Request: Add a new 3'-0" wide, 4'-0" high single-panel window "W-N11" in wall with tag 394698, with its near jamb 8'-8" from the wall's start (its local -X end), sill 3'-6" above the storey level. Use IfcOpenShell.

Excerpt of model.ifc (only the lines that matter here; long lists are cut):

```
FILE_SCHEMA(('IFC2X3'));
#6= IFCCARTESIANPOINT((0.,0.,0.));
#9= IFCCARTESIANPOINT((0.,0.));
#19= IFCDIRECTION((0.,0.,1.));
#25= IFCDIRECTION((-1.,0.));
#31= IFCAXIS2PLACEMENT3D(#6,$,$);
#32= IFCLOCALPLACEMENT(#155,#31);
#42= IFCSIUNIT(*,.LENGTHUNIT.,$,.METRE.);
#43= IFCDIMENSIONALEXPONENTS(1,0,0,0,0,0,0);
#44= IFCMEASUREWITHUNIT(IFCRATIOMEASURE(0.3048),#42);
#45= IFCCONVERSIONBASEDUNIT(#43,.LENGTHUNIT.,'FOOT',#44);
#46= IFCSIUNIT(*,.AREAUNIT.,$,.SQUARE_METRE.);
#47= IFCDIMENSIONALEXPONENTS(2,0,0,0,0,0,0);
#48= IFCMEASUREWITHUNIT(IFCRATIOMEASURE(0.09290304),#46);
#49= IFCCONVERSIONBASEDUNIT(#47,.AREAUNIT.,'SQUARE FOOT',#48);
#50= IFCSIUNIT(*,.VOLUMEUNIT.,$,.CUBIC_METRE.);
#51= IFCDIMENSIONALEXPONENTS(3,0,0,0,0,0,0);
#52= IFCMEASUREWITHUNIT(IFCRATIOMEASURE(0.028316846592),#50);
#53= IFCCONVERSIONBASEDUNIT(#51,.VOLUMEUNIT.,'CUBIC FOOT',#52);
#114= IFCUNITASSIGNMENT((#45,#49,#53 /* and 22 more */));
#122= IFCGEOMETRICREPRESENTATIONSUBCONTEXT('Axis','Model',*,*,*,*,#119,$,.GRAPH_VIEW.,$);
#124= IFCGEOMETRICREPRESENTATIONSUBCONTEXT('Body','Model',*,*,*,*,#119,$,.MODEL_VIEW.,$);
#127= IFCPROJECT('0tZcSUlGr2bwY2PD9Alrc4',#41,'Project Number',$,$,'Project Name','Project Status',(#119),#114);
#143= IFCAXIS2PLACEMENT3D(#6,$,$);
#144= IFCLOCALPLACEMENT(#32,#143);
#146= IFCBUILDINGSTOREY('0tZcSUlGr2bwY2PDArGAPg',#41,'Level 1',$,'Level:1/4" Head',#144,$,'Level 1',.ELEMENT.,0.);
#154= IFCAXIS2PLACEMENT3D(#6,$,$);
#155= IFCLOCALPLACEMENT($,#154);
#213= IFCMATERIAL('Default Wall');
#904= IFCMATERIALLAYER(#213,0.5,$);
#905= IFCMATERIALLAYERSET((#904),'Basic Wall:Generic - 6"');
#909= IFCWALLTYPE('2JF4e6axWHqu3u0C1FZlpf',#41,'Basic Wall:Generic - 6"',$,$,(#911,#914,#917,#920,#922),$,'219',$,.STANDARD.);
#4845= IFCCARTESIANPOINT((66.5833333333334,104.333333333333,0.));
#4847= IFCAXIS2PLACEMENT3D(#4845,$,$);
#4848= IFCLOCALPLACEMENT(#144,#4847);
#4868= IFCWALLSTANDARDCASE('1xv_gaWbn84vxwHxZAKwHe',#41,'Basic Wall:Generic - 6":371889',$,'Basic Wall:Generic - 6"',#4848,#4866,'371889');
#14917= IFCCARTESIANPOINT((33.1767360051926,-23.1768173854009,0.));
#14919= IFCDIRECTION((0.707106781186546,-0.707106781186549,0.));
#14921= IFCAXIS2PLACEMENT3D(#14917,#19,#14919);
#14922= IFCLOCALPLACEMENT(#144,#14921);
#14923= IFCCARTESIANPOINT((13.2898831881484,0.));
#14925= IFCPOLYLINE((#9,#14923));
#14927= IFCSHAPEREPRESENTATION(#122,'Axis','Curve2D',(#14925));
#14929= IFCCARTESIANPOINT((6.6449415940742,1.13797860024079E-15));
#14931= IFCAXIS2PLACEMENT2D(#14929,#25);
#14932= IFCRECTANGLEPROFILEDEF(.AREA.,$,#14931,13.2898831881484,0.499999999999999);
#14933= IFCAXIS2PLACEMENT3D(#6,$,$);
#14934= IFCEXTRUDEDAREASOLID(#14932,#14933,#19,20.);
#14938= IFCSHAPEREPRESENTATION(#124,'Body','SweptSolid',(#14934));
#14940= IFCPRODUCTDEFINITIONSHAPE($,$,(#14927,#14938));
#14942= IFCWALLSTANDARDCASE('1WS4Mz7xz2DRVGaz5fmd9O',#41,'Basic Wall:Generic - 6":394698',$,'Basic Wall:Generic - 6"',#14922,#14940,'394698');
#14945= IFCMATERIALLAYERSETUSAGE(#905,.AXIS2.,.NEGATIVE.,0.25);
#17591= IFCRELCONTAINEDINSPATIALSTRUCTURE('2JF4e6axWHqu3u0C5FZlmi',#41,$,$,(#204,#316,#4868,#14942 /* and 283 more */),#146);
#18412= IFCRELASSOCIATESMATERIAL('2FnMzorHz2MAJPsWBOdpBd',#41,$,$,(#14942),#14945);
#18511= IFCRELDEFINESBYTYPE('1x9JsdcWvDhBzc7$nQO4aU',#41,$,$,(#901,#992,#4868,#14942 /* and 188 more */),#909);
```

```python
import numpy as np
import ifcopenshell
import ifcopenshell.api.feature
import ifcopenshell.api.geometry
import ifcopenshell.api.root
import ifcopenshell.api.spatial
import ifcopenshell.api.type
import ifcopenshell.geom
import ifcopenshell.util.element
import ifcopenshell.util.placement
import ifcopenshell.util.representation
import ifcopenshell.util.shape
import ifcopenshell.util.unit

model = ifcopenshell.open("model.ifc")
unit_scale = ifcopenshell.util.unit.calculate_unit_scale(model)
settings = ifcopenshell.geom.settings()


def volume(element):
    """Net volume in cubic metres, openings subtracted."""
    shape = ifcopenshell.geom.create_shape(settings, element)
    return ifcopenshell.util.shape.get_volume(shape.geometry)


wall = model.by_guid("1WS4Mz7xz2DRVGaz5fmd9O")
storey = ifcopenshell.util.element.get_container(wall, ifc_class="IfcBuildingStorey")
context = ifcopenshell.util.representation.get_context(model, "Model", "Body", "MODEL_VIEW")
before = volume(wall)

width, height, from_end, sill = 0.9144, 1.2192, 2.6416, 1.0668  # metres

# The wall runs along its own X axis, and the end named is its -X end.
wall_shape = ifcopenshell.geom.create_shape(settings, wall)
x, y, z = ifcopenshell.util.shape.get_vertices(wall_shape.geometry).T
start = x.min() + from_end
face, thickness = float(y.min()), float(y.max() - y.min())
wall_matrix = ifcopenshell.util.placement.get_local_placement(wall.ObjectPlacement)
level = ifcopenshell.util.placement.get_local_placement(storey.ObjectPlacement)[2, 3]


def in_wall(x, y):
    """Placement at x, y metres in the wall's axes, at sill height."""
    matrix = wall_matrix.copy()
    matrix[:, 3] = wall_matrix @ np.array([x / unit_scale, y / unit_scale, 0.0, 1.0])
    matrix[2, 3] = level + sill / unit_scale
    return matrix


# Opening: a box that overshoots both wall faces by 50 mm.
opening = ifcopenshell.api.root.create_entity(model, ifc_class="IfcOpeningElement")
box = ifcopenshell.api.geometry.add_wall_representation(
    model, context=context, length=width, height=height, thickness=thickness + 0.1
)
ifcopenshell.api.geometry.assign_representation(model, product=opening, representation=box)
ifcopenshell.api.geometry.edit_object_placement(model, product=opening, matrix=in_wall(start, face - 0.05), is_si=False)
ifcopenshell.api.feature.add_feature(model, feature=opening, element=wall)

window = ifcopenshell.api.root.create_entity(model, ifc_class="IfcWindow", name="W-N11")
window.OverallWidth, window.OverallHeight = width / unit_scale, height / unit_scale
body = ifcopenshell.api.geometry.add_window_representation(
    model,
    context=context,
    overall_width=window.OverallWidth,
    overall_height=window.OverallHeight,
    partition_type="SINGLE_PANEL",
)
ifcopenshell.api.geometry.assign_representation(model, product=window, representation=body)
ifcopenshell.api.spatial.assign_container(model, products=[window], relating_structure=storey)
fills = ifcopenshell.api.feature.add_filling(model, opening=opening, element=window)
fills.OwnerHistory = window.OwnerHistory  # required in IFC2X3

# IFC2X3 keeps the operation on the window style.
style = ifcopenshell.api.root.create_entity(model, ifc_class="IfcWindowStyle", name="W-N11")
style.OperationType, style.ConstructionType = "SINGLE_PANEL", "NOTDEFINED"
style.ParameterTakesPrecedence = style.Sizeable = False
ifcopenshell.api.type.assign_type(model, related_objects=[window], relating_type=style)

# Centre the window in the wall's thickness.
ifcopenshell.api.geometry.edit_object_placement(model, product=window, matrix=in_wall(start, face), is_si=False)
window_shape = ifcopenshell.geom.create_shape(settings, window)
depth = ifcopenshell.util.shape.get_vertices(window_shape.geometry)[:, 1]
offset = face + thickness / 2 - (depth.min() + depth.max()) / 2
ifcopenshell.api.geometry.edit_object_placement(model, product=window, matrix=in_wall(start, offset), is_si=False)

after = volume(wall)

print(f"wall volume {before:.3f} -> {after:.3f} m3")

model.write("model_edited.ifc")
```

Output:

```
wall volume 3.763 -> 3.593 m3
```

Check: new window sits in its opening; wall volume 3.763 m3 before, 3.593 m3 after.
